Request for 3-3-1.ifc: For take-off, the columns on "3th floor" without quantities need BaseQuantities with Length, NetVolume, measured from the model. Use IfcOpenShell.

First a look at what the model holds.

```python
import ifcopenshell
import ifcopenshell.util.element
import ifcopenshell.util.unit

model = ifcopenshell.open("3-3-1.ifc")
print(model.schema)
for unit_type in ("LENGTHUNIT", "AREAUNIT", "VOLUMEUNIT"):
    print(unit_type, ifcopenshell.util.unit.calculate_unit_scale(model, unit_type))
storey = next(s for s in model.by_type("IfcBuildingStorey") if s.Name == "3th floor")
columns = [e for e in ifcopenshell.util.element.get_decomposition(storey) if e.is_a("IfcColumn")]
for e in sorted(columns, key=lambda e: e.id()):
    print(e.id(), e.is_a(), e.Name, list(ifcopenshell.util.element.get_psets(e, qtos_only=True)), sep=" | ")
```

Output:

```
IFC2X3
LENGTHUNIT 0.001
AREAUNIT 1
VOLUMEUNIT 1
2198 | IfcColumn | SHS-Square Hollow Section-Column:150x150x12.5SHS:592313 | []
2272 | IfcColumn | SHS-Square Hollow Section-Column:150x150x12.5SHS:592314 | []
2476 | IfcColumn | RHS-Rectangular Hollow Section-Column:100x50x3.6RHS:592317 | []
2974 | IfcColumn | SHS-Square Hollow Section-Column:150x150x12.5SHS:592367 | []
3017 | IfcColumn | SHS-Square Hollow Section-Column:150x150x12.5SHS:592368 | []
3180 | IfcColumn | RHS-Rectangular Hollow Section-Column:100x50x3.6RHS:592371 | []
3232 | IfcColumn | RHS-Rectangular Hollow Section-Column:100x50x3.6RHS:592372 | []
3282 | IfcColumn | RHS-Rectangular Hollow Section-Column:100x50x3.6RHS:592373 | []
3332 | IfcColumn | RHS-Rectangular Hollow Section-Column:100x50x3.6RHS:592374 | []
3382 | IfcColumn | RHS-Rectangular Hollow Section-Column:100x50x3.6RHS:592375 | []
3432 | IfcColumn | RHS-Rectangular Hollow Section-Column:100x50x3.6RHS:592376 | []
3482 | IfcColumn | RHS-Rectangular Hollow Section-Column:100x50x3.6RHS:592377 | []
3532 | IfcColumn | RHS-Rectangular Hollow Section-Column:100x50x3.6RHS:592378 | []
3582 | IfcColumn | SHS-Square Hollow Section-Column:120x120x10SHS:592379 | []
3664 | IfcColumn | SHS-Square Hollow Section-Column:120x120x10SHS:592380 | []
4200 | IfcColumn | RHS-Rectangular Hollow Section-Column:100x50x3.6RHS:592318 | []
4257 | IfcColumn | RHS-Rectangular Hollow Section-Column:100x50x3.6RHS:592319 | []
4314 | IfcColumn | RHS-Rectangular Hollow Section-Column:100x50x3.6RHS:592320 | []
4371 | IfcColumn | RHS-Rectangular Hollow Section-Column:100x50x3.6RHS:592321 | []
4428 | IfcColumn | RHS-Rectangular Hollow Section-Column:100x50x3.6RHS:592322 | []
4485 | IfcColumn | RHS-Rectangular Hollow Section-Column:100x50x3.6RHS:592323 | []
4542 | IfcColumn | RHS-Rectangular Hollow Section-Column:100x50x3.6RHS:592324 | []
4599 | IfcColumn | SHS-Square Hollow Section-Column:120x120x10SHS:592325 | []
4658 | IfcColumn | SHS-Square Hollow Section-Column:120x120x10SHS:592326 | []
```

```python
import ifcopenshell
import ifcopenshell.api.pset
import ifcopenshell.geom
import ifcopenshell.util.element
import ifcopenshell.util.shape
import ifcopenshell.util.unit

model = ifcopenshell.open("3-3-1.ifc")
unit_scale = ifcopenshell.util.unit.calculate_unit_scale(model)
volume_scale = ifcopenshell.util.unit.calculate_unit_scale(model, "VOLUMEUNIT")
settings = ifcopenshell.geom.settings()

storey = next(s for s in model.by_type("IfcBuildingStorey") if s.Name == "3th floor")
columns = [e for e in ifcopenshell.util.element.get_decomposition(storey) if e.is_a("IfcColumn")]

for e in sorted(columns, key=lambda e: e.id()):
    if ifcopenshell.util.element.get_psets(e, qtos_only=True, should_inherit=False):
        continue
    # Geometry comes back in metres, in the element's own axes.
    shape = ifcopenshell.geom.create_shape(settings, e)
    values = {
        "Length": ifcopenshell.util.shape.get_z(shape.geometry) / unit_scale,
        "NetVolume": ifcopenshell.util.shape.get_volume(shape.geometry) / volume_scale,
    }
    qto = ifcopenshell.api.pset.add_qto(model, product=e, name="BaseQuantities")
    ifcopenshell.api.pset.edit_qto(model, qto=qto, properties=values)
    print(e.id(), {k: round(v, 3) for k, v in values.items()})

model.write("3-3-1_rev.ifc")
```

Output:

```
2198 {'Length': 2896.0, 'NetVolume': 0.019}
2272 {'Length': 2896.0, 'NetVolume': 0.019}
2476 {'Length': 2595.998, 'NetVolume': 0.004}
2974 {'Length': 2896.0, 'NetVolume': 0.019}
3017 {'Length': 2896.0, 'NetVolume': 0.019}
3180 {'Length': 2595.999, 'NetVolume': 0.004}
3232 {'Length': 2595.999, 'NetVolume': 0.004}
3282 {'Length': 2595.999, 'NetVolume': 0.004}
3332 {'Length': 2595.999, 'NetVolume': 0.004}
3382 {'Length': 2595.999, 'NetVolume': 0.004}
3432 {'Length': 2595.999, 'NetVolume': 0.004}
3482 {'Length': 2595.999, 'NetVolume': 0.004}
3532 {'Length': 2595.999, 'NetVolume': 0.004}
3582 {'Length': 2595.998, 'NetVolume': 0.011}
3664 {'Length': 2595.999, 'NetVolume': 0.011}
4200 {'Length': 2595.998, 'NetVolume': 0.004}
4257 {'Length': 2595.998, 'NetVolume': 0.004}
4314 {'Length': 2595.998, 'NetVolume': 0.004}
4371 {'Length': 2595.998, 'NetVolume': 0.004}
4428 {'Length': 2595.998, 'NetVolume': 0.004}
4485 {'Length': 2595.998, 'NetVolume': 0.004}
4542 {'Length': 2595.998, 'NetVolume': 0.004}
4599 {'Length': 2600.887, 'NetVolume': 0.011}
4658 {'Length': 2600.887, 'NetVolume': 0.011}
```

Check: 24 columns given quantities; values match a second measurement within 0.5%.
